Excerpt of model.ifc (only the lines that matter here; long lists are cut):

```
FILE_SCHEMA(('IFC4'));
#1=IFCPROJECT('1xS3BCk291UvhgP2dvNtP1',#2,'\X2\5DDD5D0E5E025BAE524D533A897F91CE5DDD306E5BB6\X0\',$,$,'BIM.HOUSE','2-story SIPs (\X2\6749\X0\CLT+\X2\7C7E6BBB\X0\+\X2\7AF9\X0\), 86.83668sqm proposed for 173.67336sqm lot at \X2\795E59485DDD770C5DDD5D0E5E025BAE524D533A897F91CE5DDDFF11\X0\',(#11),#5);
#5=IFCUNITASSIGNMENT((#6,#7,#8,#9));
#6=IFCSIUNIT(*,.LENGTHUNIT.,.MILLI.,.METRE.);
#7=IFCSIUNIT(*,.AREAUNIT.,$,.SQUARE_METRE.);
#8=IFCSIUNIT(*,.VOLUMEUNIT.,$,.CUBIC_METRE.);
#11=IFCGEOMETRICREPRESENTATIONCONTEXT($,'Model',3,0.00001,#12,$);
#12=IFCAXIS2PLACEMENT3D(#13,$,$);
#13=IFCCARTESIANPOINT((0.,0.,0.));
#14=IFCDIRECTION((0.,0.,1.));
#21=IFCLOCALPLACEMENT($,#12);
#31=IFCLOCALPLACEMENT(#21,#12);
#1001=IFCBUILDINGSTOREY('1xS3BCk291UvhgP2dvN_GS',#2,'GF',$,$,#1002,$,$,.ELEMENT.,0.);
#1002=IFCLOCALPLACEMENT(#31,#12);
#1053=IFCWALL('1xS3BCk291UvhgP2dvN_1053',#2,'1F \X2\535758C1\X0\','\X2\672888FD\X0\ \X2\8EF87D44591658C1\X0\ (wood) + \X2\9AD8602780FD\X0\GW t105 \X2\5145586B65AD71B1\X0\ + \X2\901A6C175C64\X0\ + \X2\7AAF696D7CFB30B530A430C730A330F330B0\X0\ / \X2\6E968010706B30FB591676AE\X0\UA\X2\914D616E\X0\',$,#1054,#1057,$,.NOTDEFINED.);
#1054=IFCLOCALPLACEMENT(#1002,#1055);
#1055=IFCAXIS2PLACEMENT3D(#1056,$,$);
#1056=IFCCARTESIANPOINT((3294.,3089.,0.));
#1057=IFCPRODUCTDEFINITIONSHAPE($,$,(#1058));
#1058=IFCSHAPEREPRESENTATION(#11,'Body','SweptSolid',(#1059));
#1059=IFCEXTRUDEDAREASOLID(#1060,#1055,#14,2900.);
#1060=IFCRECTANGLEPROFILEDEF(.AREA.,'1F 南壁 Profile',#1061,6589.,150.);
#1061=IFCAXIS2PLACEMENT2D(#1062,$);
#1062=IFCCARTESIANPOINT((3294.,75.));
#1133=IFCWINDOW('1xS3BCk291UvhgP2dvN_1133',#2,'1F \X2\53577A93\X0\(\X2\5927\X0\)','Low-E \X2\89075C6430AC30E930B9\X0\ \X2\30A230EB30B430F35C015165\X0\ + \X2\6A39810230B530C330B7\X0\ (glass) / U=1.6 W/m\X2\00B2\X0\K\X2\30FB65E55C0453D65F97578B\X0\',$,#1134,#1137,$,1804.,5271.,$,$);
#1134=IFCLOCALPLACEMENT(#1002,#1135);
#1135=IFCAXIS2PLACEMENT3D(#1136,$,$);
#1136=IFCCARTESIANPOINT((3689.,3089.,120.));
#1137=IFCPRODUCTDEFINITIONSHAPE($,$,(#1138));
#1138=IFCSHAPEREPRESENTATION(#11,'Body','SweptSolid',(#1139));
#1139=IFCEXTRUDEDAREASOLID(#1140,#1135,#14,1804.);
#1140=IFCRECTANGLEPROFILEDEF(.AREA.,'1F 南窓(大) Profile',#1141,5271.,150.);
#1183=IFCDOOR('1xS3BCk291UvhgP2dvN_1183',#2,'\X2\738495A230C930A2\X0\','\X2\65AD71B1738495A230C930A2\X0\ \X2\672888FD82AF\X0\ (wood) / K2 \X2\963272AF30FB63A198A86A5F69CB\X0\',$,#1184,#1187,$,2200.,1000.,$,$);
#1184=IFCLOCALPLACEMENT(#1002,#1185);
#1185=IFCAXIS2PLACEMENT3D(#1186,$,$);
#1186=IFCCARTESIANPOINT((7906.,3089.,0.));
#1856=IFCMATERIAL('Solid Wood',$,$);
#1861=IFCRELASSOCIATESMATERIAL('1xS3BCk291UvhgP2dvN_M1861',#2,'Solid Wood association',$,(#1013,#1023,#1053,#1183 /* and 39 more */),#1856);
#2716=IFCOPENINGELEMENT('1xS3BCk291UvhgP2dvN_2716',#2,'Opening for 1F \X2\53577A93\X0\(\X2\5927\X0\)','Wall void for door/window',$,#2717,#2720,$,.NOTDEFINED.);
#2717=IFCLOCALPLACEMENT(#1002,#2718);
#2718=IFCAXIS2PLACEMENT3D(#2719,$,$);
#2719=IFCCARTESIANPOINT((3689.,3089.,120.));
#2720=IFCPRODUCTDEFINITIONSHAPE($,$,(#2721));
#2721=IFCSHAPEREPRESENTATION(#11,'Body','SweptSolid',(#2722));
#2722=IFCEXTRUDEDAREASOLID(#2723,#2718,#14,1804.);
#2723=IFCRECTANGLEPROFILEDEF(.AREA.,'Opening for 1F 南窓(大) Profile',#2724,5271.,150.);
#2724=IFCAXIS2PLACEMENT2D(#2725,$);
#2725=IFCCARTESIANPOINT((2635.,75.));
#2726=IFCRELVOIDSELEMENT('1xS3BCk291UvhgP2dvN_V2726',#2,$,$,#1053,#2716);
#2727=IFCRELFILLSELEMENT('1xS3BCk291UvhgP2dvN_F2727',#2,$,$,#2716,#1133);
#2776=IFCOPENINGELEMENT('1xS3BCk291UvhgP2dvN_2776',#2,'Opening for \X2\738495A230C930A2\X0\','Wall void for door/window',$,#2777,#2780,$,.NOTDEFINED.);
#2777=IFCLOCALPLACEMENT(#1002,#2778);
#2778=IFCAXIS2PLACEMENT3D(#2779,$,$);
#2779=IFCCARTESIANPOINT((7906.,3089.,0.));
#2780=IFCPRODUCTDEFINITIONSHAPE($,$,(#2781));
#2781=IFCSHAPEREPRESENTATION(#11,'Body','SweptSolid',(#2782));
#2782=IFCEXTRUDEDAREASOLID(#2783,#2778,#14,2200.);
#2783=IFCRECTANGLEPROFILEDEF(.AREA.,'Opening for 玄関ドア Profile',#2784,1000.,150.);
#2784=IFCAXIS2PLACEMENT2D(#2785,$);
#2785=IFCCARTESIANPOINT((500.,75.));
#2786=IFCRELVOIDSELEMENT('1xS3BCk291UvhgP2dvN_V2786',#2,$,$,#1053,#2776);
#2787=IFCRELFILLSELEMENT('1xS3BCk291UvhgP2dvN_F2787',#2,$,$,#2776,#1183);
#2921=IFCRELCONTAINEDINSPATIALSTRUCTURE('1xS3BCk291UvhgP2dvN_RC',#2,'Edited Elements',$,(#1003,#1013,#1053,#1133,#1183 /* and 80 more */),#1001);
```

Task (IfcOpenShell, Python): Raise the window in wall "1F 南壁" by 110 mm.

```python
import numpy as np
import ifcopenshell
import ifcopenshell.api.geometry
import ifcopenshell.util.placement
import ifcopenshell.util.unit

model = ifcopenshell.open("model.ifc")
unit_scale = ifcopenshell.util.unit.calculate_unit_scale(model)

window = model.by_id(1133)
opening = window.FillsVoids[0].RelatingOpeningElement
dz = 110.0

shift = np.array([0.0, 0.0, dz])
# The window is not placed relative to its opening, so move both.
for product in (opening, window):
    matrix = ifcopenshell.util.placement.get_local_placement(product.ObjectPlacement)
    matrix[:3, 3] += shift
    ifcopenshell.api.geometry.edit_object_placement(model, product=product, matrix=matrix, is_si=False)

print(f"moved by {dz * unit_scale:+.3f} m")

model.write("model-out.ifc")
```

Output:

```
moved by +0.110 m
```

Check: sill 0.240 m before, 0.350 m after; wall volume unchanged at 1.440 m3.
